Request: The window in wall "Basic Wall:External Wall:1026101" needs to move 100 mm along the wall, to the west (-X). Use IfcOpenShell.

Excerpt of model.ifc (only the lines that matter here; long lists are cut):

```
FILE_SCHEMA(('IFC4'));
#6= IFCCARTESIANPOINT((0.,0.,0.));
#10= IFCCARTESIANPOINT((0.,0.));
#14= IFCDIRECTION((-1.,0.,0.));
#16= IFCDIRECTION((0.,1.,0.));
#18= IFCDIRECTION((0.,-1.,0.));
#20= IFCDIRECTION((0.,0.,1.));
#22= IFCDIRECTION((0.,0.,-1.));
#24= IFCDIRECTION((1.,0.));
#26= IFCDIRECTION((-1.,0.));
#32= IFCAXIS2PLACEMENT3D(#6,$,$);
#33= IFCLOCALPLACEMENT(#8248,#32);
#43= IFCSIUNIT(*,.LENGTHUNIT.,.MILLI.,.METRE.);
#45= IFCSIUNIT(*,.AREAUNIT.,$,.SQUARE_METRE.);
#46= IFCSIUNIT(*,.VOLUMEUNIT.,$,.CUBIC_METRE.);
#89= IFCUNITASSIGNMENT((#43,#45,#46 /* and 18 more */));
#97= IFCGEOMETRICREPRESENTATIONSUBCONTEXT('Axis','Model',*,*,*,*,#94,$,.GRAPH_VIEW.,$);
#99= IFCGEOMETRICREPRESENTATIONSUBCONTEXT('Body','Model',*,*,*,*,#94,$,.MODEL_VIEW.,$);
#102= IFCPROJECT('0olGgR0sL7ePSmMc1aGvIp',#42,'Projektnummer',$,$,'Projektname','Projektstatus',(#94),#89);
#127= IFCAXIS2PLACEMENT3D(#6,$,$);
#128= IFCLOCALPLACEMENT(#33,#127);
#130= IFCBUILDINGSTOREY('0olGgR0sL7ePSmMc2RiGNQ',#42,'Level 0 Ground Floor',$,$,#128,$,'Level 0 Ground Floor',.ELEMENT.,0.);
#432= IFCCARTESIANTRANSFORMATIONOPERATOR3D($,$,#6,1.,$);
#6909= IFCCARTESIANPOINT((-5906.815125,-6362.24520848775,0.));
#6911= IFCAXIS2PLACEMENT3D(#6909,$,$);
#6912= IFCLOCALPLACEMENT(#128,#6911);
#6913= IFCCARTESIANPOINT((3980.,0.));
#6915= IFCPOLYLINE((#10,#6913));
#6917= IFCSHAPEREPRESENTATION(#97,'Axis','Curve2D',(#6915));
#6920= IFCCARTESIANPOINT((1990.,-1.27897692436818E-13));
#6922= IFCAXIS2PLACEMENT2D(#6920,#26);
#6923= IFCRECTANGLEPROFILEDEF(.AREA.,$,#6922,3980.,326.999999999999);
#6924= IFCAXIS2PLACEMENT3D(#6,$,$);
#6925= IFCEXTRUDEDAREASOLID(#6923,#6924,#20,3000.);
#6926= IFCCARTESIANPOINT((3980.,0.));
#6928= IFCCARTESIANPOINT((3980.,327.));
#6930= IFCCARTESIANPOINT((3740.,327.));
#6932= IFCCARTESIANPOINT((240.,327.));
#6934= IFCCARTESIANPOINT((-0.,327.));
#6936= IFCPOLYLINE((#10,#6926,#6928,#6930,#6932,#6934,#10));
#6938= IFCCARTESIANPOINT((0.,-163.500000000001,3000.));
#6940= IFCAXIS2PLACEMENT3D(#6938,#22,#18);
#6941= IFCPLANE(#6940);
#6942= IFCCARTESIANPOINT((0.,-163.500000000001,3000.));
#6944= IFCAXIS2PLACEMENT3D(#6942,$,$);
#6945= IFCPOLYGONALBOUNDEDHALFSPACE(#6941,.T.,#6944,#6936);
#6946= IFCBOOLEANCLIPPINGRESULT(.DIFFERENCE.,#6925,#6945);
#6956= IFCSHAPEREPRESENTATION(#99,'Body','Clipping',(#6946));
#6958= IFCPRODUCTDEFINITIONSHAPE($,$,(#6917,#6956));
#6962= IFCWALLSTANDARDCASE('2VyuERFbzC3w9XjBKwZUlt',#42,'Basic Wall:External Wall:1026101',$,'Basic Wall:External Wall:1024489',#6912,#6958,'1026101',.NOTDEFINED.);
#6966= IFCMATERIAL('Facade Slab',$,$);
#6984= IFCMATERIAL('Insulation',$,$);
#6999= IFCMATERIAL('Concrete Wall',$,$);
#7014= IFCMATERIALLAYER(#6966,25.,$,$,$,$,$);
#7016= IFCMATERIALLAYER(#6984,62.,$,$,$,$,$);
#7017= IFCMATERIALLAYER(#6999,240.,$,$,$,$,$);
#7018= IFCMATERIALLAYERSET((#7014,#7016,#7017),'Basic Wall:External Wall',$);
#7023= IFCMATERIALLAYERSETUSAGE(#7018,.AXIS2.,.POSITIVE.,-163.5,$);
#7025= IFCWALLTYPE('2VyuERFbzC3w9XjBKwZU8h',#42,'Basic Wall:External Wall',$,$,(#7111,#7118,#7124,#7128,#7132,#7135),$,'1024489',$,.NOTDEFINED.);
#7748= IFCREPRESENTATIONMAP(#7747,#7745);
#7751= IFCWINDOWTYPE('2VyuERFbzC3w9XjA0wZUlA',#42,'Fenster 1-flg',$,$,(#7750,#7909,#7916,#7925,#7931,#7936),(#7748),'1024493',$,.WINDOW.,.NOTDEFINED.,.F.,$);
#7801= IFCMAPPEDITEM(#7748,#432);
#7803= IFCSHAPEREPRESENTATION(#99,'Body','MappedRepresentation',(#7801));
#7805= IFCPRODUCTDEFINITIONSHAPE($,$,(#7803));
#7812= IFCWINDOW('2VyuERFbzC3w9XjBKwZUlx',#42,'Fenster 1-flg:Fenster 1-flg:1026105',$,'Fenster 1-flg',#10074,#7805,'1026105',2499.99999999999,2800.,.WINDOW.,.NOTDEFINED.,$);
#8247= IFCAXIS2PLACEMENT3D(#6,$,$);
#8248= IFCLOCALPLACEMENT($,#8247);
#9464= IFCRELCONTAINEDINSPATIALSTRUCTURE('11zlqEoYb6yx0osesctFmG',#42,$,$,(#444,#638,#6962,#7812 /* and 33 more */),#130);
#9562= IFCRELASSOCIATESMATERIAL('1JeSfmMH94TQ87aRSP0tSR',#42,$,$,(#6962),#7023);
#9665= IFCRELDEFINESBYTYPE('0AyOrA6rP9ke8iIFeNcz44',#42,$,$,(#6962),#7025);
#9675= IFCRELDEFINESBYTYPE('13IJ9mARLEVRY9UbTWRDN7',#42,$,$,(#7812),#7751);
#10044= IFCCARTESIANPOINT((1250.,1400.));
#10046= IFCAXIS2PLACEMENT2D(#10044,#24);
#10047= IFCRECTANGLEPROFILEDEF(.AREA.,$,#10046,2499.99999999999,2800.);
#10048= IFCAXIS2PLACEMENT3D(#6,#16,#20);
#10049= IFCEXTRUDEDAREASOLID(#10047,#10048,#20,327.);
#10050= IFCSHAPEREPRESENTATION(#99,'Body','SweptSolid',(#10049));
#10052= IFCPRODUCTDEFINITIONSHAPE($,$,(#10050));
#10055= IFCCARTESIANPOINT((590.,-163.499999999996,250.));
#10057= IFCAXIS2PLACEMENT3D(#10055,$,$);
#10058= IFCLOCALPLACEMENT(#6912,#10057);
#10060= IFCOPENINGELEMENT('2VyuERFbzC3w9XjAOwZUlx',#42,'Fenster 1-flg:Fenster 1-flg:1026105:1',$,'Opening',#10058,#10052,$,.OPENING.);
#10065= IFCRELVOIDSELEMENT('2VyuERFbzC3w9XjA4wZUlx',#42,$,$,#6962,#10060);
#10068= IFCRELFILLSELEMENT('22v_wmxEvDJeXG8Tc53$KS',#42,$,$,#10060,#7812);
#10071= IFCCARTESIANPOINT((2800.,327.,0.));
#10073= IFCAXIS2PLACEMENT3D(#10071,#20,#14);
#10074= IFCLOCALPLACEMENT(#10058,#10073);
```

```python
import ifcopenshell
import ifcopenshell.api.geometry
import ifcopenshell.util.placement
import ifcopenshell.util.unit

model = ifcopenshell.open("model.ifc")
unit_scale = ifcopenshell.util.unit.calculate_unit_scale(model)

window = model.by_guid("2VyuERFbzC3w9XjBKwZUlx")
opening = window.FillsVoids[0].RelatingOpeningElement
wall = opening.VoidsElements[0].RelatingBuildingElement

wall_matrix = ifcopenshell.util.placement.get_local_placement(wall.ObjectPlacement)
shift = wall_matrix[:3, 0] * -0.1 / unit_scale
before = ifcopenshell.util.placement.get_local_placement(window.ObjectPlacement)[:3, 3].copy()

# The window is placed relative to its opening, so it follows when the opening moves.
matrix = ifcopenshell.util.placement.get_local_placement(opening.ObjectPlacement)
matrix[:3, 3] += shift
ifcopenshell.api.geometry.edit_object_placement(
    model, product=opening, matrix=matrix, is_si=False, should_transform_children=True
)

after = ifcopenshell.util.placement.get_local_placement(window.ObjectPlacement)[:3, 3]
print("window moved by", (after - before).round(3) + 0.0)

model.write("model_edited.ifc")
```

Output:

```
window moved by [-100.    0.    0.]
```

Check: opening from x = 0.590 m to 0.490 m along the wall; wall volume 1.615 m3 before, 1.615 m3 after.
